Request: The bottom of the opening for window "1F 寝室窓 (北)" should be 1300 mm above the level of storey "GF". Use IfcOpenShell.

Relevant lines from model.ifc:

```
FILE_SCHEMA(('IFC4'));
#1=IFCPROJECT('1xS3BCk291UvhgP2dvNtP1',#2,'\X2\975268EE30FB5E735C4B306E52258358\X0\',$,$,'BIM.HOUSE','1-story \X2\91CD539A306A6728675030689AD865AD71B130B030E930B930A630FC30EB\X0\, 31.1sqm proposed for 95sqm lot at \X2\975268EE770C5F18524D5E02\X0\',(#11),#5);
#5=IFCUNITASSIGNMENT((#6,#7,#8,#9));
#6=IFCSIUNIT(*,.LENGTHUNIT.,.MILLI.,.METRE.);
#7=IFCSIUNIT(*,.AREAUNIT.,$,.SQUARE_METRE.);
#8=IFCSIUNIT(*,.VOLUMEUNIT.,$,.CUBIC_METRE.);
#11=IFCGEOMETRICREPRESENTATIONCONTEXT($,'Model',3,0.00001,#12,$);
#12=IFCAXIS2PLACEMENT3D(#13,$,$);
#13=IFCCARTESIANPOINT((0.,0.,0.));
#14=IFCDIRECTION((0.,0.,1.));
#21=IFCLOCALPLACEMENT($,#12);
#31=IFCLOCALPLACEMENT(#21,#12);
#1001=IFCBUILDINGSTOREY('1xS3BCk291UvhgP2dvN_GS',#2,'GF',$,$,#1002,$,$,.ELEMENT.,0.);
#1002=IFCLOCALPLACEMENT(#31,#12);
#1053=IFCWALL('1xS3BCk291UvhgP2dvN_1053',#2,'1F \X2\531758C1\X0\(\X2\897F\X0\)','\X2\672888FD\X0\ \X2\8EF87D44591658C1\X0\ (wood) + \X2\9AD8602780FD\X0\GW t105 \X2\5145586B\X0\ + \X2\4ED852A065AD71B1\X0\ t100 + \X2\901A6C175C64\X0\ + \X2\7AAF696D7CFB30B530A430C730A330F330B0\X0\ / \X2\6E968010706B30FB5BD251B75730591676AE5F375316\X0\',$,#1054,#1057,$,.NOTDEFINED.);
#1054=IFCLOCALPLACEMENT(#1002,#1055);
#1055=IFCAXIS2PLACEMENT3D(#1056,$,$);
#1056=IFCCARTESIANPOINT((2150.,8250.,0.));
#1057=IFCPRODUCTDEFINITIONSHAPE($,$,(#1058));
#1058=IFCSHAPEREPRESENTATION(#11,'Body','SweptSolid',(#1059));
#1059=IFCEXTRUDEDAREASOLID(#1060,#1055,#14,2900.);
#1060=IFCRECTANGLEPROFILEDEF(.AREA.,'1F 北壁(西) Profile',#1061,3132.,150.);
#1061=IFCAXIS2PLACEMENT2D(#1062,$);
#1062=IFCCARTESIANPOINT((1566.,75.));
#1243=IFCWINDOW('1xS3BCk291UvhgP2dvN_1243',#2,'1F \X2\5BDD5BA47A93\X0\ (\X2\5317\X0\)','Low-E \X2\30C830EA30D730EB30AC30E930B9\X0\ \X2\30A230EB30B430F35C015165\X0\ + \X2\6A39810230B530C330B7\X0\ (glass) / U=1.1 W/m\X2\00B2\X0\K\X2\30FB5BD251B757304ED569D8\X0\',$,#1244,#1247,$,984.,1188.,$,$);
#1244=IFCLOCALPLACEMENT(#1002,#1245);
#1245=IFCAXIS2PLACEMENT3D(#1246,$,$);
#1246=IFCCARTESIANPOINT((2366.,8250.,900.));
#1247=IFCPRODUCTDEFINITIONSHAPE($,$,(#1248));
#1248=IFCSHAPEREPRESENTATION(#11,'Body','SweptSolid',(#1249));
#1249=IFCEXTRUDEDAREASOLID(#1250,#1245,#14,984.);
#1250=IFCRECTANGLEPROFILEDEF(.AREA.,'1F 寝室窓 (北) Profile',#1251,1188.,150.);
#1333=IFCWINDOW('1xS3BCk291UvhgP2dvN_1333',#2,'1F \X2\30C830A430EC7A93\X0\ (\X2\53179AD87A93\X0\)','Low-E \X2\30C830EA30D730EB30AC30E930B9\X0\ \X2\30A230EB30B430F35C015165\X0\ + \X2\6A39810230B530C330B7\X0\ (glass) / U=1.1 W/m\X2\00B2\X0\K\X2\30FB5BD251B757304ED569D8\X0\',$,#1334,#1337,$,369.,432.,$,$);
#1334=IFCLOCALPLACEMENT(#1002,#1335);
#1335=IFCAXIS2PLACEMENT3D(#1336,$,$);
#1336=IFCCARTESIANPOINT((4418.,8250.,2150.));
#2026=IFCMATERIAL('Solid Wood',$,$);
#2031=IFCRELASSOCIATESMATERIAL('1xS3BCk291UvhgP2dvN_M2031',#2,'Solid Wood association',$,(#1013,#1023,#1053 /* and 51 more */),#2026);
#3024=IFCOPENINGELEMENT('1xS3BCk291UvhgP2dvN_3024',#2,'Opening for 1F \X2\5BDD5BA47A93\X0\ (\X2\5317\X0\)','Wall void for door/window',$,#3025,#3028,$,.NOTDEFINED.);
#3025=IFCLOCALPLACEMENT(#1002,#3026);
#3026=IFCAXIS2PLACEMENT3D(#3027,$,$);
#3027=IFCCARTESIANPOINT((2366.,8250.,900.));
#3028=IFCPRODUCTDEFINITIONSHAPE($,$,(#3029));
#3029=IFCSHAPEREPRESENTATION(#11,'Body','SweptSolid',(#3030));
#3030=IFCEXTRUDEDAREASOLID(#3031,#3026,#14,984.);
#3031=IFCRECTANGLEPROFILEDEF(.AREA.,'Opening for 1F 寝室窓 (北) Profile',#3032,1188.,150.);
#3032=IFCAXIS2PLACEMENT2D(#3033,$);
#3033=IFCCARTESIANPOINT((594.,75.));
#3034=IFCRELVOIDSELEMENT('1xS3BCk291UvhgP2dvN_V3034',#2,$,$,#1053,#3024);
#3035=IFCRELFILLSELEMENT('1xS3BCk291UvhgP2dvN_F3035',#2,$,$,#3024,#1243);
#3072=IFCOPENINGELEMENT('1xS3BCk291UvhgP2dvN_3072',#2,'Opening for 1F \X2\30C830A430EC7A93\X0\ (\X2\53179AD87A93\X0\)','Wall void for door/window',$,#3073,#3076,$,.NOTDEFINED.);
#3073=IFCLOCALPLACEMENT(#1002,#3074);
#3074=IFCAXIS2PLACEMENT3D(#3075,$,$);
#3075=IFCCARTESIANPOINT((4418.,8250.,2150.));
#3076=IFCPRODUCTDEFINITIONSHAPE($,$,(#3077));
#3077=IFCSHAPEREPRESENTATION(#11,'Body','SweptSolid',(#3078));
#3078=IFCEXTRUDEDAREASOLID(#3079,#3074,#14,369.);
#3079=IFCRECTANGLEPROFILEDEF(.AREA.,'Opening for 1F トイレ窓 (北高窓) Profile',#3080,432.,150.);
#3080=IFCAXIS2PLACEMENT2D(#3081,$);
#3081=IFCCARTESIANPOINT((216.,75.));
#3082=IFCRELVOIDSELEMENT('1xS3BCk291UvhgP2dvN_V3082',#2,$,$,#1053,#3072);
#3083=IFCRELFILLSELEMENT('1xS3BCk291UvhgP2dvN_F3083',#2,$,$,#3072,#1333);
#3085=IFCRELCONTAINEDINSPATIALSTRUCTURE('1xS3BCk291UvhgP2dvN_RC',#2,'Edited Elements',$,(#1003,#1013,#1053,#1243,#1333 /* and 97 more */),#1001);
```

```python
import numpy as np
import ifcopenshell
import ifcopenshell.api.geometry
import ifcopenshell.geom
import ifcopenshell.util.element
import ifcopenshell.util.placement
import ifcopenshell.util.shape
import ifcopenshell.util.unit

model = ifcopenshell.open("model.ifc")
unit_scale = ifcopenshell.util.unit.calculate_unit_scale(model)

window = model.by_guid("1xS3BCk291UvhgP2dvN_1243")
opening = window.FillsVoids[0].RelatingOpeningElement
storey = ifcopenshell.util.element.get_container(window, ifc_class="IfcBuildingStorey")
level = ifcopenshell.util.placement.get_local_placement(storey.ObjectPlacement)[2, 3]

# The opening's origin need not be at the sill, so measure its lowest point.
shape = ifcopenshell.geom.create_shape(ifcopenshell.geom.settings(), opening)
bottom = ifcopenshell.util.shape.get_shape_bottom_elevation(shape, shape.geometry) / unit_scale
dz = level + 1.3 / unit_scale - bottom

shift = np.array([0.0, 0.0, dz])
# The window is not placed relative to its opening, so move both.
for product in (opening, window):
    matrix = ifcopenshell.util.placement.get_local_placement(product.ObjectPlacement)
    matrix[:3, 3] += shift
    ifcopenshell.api.geometry.edit_object_placement(model, product=product, matrix=matrix, is_si=False)

print(f"moved by {dz * unit_scale:+.3f} m")

model.write("model_rev.ifc")
```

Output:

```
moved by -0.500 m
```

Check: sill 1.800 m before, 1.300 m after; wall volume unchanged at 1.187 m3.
